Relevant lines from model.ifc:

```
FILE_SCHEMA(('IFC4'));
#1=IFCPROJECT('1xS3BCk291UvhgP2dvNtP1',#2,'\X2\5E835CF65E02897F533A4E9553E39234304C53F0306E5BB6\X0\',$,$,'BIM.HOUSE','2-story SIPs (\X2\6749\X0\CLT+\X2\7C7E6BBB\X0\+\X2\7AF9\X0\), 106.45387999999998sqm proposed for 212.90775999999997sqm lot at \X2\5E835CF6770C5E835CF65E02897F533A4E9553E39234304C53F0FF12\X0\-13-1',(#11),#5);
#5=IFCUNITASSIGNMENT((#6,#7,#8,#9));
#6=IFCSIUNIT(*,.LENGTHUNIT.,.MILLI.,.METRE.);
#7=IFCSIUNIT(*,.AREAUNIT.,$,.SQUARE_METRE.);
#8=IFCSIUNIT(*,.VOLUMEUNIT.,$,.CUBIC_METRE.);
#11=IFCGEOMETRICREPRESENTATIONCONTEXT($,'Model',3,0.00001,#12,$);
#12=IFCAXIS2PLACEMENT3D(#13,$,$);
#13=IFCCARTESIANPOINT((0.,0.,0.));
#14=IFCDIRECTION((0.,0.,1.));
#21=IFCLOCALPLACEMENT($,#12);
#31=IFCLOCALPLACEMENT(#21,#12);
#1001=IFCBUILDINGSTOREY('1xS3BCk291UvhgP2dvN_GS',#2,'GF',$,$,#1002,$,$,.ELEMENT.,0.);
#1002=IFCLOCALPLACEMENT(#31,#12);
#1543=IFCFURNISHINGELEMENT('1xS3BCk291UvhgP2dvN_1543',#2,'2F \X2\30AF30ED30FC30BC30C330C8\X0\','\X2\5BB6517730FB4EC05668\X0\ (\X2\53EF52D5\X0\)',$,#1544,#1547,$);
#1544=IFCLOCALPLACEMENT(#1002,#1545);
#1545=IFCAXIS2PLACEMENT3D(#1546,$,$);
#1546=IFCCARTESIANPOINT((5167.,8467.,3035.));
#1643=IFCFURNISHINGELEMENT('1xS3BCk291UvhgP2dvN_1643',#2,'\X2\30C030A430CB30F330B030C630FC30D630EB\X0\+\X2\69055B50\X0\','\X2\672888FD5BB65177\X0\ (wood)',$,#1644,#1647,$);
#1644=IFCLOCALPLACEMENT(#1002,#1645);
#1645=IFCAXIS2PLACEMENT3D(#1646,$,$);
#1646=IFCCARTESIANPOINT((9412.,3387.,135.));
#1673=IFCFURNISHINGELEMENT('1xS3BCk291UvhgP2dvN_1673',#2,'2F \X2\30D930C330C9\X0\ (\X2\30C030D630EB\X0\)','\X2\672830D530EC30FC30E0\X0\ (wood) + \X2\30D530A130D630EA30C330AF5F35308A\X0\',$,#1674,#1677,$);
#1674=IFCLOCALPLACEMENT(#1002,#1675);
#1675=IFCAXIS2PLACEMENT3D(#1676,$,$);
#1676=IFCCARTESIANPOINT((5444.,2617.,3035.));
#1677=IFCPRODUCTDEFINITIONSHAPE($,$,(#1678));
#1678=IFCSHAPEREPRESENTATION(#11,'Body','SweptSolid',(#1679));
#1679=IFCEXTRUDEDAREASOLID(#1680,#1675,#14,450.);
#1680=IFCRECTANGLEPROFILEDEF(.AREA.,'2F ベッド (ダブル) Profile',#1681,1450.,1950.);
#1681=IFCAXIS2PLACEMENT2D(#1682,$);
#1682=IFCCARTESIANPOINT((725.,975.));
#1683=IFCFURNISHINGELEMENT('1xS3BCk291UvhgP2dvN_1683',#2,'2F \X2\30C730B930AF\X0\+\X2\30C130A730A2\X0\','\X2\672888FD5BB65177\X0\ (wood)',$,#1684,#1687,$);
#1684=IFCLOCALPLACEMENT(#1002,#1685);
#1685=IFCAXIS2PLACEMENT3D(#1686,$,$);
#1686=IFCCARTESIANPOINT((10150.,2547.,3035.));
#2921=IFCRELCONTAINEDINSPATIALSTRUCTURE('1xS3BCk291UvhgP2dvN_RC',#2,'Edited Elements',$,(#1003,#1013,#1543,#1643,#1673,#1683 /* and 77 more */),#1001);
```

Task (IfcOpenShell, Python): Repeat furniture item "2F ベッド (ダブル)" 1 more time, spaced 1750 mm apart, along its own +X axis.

```python
import ifcopenshell
import ifcopenshell.api.geometry
import ifcopenshell.api.root
import ifcopenshell.util.element
import ifcopenshell.util.placement

model = ifcopenshell.open("model.ifc")


def reuse_history(source, copy):
    """copy_class also copies each property set's owner history, people and application; keep the originals."""
    for rel in copy.IsDefinedBy:
        if rel.is_a("IfcRelDefinesByProperties") and (history := rel.RelatingPropertyDefinition.OwnerHistory):
            rel.RelatingPropertyDefinition.OwnerHistory = source.OwnerHistory
            ifcopenshell.util.element.remove_deep2(model, history)


source = model.by_guid("1xS3BCk291UvhgP2dvN_1673")
base = ifcopenshell.util.placement.get_local_placement(source.ObjectPlacement)
step = base[:3, 0] * 1750.0

for i in range(1, 2):
    copy = ifcopenshell.api.root.copy_class(model, product=source)
    copy.Representation = ifcopenshell.util.element.copy_deep(
        model, source.Representation, exclude=["IfcGeometricRepresentationContext", "IfcRepresentationMap"]
    )
    reuse_history(source, copy)
    matrix = base.copy()
    matrix[:3, 3] += i * step
    print("added at", matrix[:3, 3].round(3) + 0.0)
    ifcopenshell.api.geometry.edit_object_placement(model, product=copy, matrix=matrix, is_si=False)

model.write("model_edited.ifc")
```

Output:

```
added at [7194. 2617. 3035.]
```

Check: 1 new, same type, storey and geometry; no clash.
